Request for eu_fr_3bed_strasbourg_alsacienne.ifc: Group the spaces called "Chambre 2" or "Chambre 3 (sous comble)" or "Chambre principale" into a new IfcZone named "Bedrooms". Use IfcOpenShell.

First a look at what the model holds.

```python
import ifcopenshell

model = ifcopenshell.open("eu_fr_3bed_strasbourg_alsacienne.ifc")
print(model.schema)
seen = {}
for space in model.by_type("IfcSpace"):
    seen[space.LongName] = seen.get(space.LongName, 0) + 1
for name, count in sorted(seen.items(), key=str):
    print(count, "x", name)
print("zones:", [z.Name for z in model.by_type("IfcZone")][:20])
```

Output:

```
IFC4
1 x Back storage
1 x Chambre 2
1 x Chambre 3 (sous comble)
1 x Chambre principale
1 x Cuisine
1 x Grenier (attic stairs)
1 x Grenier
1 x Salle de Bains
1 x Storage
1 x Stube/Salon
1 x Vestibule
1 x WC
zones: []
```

```python
import ifcopenshell
import ifcopenshell.api.group
import ifcopenshell.api.root

model = ifcopenshell.open("eu_fr_3bed_strasbourg_alsacienne.ifc")

names = {"Chambre 2", "Chambre 3 (sous comble)", "Chambre principale"}
spaces = [s for s in model.by_type("IfcSpace") if s.LongName in names]

zone = ifcopenshell.api.root.create_entity(model, ifc_class="IfcZone", name="Bedrooms")
ifcopenshell.api.group.assign_group(model, products=spaces, group=zone)
print(len(spaces), "spaces in", zone.Name)

model.write("eu_fr_3bed_strasbourg_alsacienne-out.ifc")
```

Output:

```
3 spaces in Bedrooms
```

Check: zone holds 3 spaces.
